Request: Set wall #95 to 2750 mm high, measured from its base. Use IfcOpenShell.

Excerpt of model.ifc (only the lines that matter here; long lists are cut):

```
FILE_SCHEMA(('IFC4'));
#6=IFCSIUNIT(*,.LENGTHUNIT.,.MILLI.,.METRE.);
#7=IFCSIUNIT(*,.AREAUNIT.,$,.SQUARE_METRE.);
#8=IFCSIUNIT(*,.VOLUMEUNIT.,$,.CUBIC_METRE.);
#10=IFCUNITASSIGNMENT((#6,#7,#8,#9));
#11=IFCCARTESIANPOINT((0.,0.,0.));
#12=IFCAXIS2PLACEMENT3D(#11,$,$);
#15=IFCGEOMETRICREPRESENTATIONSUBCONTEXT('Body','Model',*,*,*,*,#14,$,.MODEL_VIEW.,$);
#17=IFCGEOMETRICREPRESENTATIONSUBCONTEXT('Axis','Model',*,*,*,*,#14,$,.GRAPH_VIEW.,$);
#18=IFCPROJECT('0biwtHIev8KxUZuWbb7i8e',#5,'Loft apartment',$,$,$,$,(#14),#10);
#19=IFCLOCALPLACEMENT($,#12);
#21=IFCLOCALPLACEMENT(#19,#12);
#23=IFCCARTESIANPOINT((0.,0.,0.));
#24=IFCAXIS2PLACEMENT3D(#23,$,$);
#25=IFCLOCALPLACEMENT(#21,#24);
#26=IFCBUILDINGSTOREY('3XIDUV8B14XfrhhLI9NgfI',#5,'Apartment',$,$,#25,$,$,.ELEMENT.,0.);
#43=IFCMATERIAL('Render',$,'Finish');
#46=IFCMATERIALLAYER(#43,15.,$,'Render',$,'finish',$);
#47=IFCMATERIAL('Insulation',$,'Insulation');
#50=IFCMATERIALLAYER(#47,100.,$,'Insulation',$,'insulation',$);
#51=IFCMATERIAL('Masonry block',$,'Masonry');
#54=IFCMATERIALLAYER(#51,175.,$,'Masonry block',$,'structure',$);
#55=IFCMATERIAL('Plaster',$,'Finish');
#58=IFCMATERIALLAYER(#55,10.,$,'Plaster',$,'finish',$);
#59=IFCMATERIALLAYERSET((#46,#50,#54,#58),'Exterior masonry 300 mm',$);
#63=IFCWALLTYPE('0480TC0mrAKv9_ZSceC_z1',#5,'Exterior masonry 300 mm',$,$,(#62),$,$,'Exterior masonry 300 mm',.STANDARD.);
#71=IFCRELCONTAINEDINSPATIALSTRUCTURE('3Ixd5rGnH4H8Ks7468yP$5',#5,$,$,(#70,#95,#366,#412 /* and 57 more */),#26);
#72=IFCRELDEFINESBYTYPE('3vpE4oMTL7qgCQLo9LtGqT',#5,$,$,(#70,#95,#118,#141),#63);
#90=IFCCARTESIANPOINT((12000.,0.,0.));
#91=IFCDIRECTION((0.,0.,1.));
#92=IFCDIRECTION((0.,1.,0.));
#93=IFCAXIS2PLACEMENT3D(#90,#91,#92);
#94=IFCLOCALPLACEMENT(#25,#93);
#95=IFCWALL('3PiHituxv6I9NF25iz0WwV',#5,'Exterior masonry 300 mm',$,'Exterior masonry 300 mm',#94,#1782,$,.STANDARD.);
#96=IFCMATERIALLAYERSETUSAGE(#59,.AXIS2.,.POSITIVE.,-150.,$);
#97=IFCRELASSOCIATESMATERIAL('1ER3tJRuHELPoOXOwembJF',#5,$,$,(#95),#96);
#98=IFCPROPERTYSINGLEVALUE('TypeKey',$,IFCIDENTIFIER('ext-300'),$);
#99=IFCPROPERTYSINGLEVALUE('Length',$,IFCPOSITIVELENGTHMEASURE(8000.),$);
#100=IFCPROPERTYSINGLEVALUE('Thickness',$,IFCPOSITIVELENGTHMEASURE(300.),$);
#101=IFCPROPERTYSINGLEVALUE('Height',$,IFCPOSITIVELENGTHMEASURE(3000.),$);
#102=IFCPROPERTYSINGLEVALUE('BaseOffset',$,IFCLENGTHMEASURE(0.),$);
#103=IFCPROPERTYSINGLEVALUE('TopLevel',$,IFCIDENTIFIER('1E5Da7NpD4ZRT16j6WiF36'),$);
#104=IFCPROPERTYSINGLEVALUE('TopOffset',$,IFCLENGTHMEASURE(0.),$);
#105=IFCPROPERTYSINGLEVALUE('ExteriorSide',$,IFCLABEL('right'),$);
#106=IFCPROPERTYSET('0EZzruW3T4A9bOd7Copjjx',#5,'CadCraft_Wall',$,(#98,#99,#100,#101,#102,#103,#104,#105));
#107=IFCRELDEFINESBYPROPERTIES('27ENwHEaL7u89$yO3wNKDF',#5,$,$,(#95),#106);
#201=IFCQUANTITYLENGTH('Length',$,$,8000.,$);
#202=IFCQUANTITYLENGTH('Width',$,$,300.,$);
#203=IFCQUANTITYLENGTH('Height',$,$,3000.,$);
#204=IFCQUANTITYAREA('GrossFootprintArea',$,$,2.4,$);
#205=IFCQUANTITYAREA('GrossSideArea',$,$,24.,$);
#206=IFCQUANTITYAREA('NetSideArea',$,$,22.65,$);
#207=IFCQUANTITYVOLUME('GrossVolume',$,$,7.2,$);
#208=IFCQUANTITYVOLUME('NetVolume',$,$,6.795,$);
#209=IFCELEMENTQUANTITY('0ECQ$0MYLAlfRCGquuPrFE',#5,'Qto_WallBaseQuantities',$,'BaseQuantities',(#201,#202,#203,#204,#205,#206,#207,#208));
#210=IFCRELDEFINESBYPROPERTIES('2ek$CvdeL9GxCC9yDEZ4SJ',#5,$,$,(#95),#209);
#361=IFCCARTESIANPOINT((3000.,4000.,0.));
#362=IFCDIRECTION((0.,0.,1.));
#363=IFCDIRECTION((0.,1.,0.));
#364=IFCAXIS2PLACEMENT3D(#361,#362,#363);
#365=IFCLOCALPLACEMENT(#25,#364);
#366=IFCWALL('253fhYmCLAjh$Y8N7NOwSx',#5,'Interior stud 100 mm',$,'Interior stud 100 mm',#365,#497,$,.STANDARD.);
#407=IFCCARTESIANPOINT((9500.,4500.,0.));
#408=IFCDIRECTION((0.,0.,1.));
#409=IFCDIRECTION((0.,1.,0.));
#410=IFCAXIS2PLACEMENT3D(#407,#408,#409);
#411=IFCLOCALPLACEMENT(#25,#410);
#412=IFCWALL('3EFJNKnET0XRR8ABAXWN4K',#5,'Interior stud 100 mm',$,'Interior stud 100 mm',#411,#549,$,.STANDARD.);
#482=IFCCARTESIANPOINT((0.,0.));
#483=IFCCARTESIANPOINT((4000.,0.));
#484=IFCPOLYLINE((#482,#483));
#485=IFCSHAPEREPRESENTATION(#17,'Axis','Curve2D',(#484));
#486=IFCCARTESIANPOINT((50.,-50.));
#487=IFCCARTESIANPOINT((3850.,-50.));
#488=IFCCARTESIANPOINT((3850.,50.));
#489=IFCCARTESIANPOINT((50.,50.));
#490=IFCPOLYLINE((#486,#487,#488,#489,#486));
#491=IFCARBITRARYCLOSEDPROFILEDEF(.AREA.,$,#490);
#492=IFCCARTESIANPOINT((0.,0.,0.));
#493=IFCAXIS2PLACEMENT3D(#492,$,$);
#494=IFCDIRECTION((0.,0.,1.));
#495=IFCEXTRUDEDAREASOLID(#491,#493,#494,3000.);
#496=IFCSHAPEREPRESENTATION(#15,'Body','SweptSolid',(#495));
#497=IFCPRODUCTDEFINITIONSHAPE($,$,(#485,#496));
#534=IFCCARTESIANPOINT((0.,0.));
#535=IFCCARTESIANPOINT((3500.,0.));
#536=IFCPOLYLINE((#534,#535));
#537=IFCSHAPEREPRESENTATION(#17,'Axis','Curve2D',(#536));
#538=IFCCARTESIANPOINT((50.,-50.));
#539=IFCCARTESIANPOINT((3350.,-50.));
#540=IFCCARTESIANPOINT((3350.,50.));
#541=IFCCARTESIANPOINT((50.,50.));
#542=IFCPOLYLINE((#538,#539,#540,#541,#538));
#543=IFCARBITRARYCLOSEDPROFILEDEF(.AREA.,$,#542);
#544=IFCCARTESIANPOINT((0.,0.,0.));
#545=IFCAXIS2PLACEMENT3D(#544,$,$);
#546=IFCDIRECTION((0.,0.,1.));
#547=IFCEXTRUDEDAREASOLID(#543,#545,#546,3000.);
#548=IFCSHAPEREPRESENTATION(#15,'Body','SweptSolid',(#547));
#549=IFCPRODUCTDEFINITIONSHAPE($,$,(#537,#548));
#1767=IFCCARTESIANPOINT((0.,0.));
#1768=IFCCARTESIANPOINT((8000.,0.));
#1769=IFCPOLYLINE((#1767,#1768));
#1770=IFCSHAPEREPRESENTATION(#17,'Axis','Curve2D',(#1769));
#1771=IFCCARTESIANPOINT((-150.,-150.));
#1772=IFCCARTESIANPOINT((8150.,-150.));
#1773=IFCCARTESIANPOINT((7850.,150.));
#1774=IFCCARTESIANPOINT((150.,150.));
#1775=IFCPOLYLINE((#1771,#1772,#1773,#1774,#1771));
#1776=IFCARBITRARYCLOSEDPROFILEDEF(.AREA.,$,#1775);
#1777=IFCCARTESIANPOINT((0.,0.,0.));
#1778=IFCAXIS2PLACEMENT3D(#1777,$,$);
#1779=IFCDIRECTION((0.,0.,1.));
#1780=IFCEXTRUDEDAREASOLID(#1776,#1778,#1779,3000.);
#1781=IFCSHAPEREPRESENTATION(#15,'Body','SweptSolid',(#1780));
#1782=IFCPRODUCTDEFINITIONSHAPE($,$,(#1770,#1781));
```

```python
import ifcopenshell
import ifcopenshell.api.pset
import ifcopenshell.geom
import ifcopenshell.util.element
import ifcopenshell.util.representation
import ifcopenshell.util.shape
import ifcopenshell.util.unit

model = ifcopenshell.open("model.ifc")
unit_scale = ifcopenshell.util.unit.calculate_unit_scale(model)
area_scale = ifcopenshell.util.unit.calculate_unit_scale(model, "AREAUNIT")
volume_scale = ifcopenshell.util.unit.calculate_unit_scale(model, "VOLUMEUNIT")
settings = ifcopenshell.geom.settings()


def volume(element):
    """Net volume in cubic metres, openings subtracted."""
    shape = ifcopenshell.geom.create_shape(settings, element)
    return ifcopenshell.util.shape.get_volume(shape.geometry)


wall = model.by_guid("3PiHituxv6I9NF25iz0WwV")
before = volume(wall)

body = ifcopenshell.util.representation.get_representation(wall, "Model", "Body")
solid = body.Items[0]
old_height = solid.Depth
solid.Depth = 2.75 / unit_scale
after = volume(wall)
thickness = 0.3  # wall thickness in metres

# Update the stored height, areas and volumes.
pset = model.by_id(ifcopenshell.util.element.get_pset(wall, "CadCraft_Wall", should_inherit=False)["id"])
ifcopenshell.api.pset.edit_pset(model, pset=pset, properties={
    "Height": model.create_entity("IfcPositiveLengthMeasure", solid.Depth),
})
qto = model.by_id(ifcopenshell.util.element.get_pset(wall, "Qto_WallBaseQuantities", should_inherit=False)["id"])
ifcopenshell.api.pset.edit_qto(model, qto=qto, properties={
    "Height": solid.Depth,
    "GrossSideArea": ifcopenshell.util.element.get_pset(wall, "Qto_WallBaseQuantities", "GrossSideArea") * solid.Depth / old_height,
    "NetSideArea": after / thickness / area_scale,
    "GrossVolume": ifcopenshell.util.element.get_pset(wall, "Qto_WallBaseQuantities", "GrossVolume") * solid.Depth / old_height,
    "NetVolume": after / volume_scale,
})

print(f"height {old_height:g} -> {solid.Depth:g}, volume {before:.3f} -> {after:.3f} m3")

model.write("model_v2.ifc")
```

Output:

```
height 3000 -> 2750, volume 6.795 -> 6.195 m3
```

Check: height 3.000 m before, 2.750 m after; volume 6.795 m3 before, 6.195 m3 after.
